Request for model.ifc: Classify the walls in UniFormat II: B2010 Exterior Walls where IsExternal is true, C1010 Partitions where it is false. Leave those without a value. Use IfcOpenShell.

First a look at what the model holds.

```python
import ifcopenshell
import ifcopenshell.util.element

model = ifcopenshell.open("model.ifc")
print(model.schema)
print("classifications:", [c.Name for c in model.by_type("IfcClassification")])
values = [ifcopenshell.util.element.get_pset(e, "Pset_WallCommon", "IsExternal") for e in model.by_type("IfcWall")]
for value in (True, False, None):
    print("IsExternal", value, values.count(value))
```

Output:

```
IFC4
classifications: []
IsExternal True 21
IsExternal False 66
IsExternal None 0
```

```python
import ifcopenshell
import ifcopenshell.api.classification
import ifcopenshell.util.element

model = ifcopenshell.open("model.ifc")

system = ifcopenshell.api.classification.add_classification(model, classification="UniFormat II")

walls = model.by_type("IfcWall")
external = {e: ifcopenshell.util.element.get_pset(e, "Pset_WallCommon", "IsExternal") for e in walls}
for flag, code, name in ((True, "B2010", "Exterior Walls"), (False, "C1010", "Partitions")):
    products = [e for e in walls if external[e] is flag]
    ifcopenshell.api.classification.add_reference(
        model, products=products, classification=system, identification=code, name=name
    )
    print(code, len(products))

model.write("model_edited.ifc")
```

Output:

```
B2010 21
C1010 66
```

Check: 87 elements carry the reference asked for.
